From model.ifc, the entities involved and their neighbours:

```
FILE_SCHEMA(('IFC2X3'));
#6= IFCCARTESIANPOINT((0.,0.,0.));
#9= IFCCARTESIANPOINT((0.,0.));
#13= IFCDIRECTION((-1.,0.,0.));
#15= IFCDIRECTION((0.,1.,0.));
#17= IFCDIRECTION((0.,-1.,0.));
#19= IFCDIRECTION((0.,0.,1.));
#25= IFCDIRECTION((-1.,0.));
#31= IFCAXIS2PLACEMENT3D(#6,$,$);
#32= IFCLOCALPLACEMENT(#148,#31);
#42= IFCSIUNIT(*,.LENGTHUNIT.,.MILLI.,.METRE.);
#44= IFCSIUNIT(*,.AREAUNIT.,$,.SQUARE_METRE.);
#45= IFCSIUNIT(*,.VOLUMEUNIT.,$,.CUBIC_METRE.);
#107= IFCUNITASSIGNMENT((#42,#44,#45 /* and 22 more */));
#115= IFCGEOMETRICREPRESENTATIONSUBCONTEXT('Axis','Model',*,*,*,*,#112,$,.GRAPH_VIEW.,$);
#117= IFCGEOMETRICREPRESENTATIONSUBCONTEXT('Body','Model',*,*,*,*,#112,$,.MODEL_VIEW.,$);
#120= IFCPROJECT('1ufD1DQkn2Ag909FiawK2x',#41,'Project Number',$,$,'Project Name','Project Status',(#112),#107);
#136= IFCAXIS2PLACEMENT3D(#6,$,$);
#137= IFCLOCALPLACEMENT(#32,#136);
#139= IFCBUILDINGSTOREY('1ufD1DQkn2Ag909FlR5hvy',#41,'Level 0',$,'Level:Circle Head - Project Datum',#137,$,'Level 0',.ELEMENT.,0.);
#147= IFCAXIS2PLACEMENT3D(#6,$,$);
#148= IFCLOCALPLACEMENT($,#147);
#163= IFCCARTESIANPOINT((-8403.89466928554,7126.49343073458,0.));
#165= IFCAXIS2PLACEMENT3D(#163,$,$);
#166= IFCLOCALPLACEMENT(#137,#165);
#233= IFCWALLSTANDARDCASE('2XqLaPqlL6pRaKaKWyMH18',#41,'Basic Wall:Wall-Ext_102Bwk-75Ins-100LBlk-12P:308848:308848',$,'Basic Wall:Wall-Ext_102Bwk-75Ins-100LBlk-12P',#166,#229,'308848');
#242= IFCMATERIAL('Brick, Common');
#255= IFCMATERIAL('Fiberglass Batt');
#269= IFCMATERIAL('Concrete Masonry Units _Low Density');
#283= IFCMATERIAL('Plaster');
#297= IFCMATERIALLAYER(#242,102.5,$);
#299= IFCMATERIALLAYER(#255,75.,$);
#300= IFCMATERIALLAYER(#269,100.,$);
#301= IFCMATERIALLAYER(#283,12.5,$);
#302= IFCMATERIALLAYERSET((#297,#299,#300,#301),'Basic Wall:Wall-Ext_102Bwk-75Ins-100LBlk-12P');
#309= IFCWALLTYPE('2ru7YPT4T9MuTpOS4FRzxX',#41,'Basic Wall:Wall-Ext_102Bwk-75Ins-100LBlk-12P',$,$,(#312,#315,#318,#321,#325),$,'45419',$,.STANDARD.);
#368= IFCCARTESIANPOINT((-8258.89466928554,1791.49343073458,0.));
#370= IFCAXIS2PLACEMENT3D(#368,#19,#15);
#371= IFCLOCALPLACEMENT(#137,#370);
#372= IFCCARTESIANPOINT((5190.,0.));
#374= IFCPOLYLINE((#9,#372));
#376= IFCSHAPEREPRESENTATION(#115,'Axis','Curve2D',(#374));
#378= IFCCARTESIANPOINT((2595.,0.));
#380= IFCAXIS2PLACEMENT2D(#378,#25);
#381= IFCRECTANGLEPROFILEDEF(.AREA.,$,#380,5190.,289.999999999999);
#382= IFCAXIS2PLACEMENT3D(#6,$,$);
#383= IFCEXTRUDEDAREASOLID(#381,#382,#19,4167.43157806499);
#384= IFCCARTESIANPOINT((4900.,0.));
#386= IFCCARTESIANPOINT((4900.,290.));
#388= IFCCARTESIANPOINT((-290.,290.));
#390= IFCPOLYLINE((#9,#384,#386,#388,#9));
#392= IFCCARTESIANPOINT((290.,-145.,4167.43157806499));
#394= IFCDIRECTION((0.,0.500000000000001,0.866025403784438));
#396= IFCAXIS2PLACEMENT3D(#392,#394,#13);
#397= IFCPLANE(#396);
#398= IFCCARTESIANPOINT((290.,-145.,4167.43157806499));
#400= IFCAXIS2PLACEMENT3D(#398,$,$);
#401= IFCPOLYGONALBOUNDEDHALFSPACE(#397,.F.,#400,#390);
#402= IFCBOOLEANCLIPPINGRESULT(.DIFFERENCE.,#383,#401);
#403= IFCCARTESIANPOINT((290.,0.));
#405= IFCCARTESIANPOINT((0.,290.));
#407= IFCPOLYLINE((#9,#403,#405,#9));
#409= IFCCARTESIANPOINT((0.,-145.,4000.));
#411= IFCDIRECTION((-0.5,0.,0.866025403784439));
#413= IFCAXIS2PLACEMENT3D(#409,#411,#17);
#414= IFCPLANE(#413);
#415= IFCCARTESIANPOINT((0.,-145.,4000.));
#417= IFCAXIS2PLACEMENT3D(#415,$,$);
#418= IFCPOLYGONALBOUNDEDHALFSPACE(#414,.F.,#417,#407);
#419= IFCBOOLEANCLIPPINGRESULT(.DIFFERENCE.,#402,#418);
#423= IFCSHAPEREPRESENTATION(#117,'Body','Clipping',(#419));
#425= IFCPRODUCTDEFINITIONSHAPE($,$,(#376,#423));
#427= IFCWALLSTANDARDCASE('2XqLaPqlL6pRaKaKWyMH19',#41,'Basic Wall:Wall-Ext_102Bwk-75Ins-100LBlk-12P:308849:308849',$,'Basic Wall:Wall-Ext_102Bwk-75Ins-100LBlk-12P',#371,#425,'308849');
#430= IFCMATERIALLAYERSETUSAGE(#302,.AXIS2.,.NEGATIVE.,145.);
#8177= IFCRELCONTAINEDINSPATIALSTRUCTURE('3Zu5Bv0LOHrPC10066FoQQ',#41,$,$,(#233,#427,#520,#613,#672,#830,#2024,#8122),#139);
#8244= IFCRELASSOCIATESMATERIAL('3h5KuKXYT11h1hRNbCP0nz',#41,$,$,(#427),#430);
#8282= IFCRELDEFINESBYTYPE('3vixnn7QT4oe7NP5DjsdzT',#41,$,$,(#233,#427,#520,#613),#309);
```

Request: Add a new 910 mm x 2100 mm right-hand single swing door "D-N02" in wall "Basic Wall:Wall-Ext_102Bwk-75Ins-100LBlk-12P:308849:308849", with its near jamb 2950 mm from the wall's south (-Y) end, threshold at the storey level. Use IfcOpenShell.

```python
import numpy as np
import ifcopenshell
import ifcopenshell.api.feature
import ifcopenshell.api.geometry
import ifcopenshell.api.root
import ifcopenshell.api.spatial
import ifcopenshell.api.type
import ifcopenshell.geom
import ifcopenshell.util.element
import ifcopenshell.util.placement
import ifcopenshell.util.representation
import ifcopenshell.util.shape
import ifcopenshell.util.unit

model = ifcopenshell.open("model.ifc")
unit_scale = ifcopenshell.util.unit.calculate_unit_scale(model)
settings = ifcopenshell.geom.settings()


def volume(element):
    """Net volume in cubic metres, openings subtracted."""
    shape = ifcopenshell.geom.create_shape(settings, element)
    return ifcopenshell.util.shape.get_volume(shape.geometry)


wall = model.by_guid("2XqLaPqlL6pRaKaKWyMH19")
storey = ifcopenshell.util.element.get_container(wall, ifc_class="IfcBuildingStorey")
context = ifcopenshell.util.representation.get_context(model, "Model", "Body", "MODEL_VIEW")
before = volume(wall)

width, height, from_end, sill = 0.91, 2.1, 2.95, 0.0  # metres

# The wall runs along its own X axis, and the end named is its -X end.
wall_shape = ifcopenshell.geom.create_shape(settings, wall)
x, y, z = ifcopenshell.util.shape.get_vertices(wall_shape.geometry).T
start = x.min() + from_end
face, thickness = float(y.min()), float(y.max() - y.min())
wall_matrix = ifcopenshell.util.placement.get_local_placement(wall.ObjectPlacement)
level = ifcopenshell.util.placement.get_local_placement(storey.ObjectPlacement)[2, 3]


def in_wall(x, y):
    """Placement at x, y metres in the wall's axes, at sill height."""
    matrix = wall_matrix.copy()
    matrix[:, 3] = wall_matrix @ np.array([x / unit_scale, y / unit_scale, 0.0, 1.0])
    matrix[2, 3] = level + sill / unit_scale
    return matrix


# Opening: a box that overshoots both wall faces by 50 mm.
opening = ifcopenshell.api.root.create_entity(model, ifc_class="IfcOpeningElement")
box = ifcopenshell.api.geometry.add_wall_representation(
    model, context=context, length=width, height=height, thickness=thickness + 0.1
)
ifcopenshell.api.geometry.assign_representation(model, product=opening, representation=box)
ifcopenshell.api.geometry.edit_object_placement(model, product=opening, matrix=in_wall(start, face - 0.05), is_si=False)
ifcopenshell.api.feature.add_feature(model, feature=opening, element=wall)

door = ifcopenshell.api.root.create_entity(model, ifc_class="IfcDoor", name="D-N02")
door.OverallWidth, door.OverallHeight = width / unit_scale, height / unit_scale
body = ifcopenshell.api.geometry.add_door_representation(
    model,
    context=context,
    overall_width=door.OverallWidth,
    overall_height=door.OverallHeight,
    operation_type="SINGLE_SWING_RIGHT",
    lining_properties={"LiningDepth": thickness / unit_scale, "ThresholdDepth": thickness / unit_scale},
)
ifcopenshell.api.geometry.assign_representation(model, product=door, representation=body)
ifcopenshell.api.spatial.assign_container(model, products=[door], relating_structure=storey)
fills = ifcopenshell.api.feature.add_filling(model, opening=opening, element=door)
fills.OwnerHistory = door.OwnerHistory  # required in IFC2X3

# IFC2X3 keeps the operation on the door style.
style = ifcopenshell.api.root.create_entity(model, ifc_class="IfcDoorStyle", name="D-N02")
style.OperationType, style.ConstructionType = "SINGLE_SWING_RIGHT", "NOTDEFINED"
style.ParameterTakesPrecedence = style.Sizeable = False
ifcopenshell.api.type.assign_type(model, related_objects=[door], relating_type=style)

# The lining spans the wall, so the door starts at the wall face.
ifcopenshell.api.geometry.edit_object_placement(model, product=door, matrix=in_wall(start, face), is_si=False)

after = volume(wall)

print(f"wall volume {before:.3f} -> {after:.3f} m3")

model.write("model_edited.ifc")
```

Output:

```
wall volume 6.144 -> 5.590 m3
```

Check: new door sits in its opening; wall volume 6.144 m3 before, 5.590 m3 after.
